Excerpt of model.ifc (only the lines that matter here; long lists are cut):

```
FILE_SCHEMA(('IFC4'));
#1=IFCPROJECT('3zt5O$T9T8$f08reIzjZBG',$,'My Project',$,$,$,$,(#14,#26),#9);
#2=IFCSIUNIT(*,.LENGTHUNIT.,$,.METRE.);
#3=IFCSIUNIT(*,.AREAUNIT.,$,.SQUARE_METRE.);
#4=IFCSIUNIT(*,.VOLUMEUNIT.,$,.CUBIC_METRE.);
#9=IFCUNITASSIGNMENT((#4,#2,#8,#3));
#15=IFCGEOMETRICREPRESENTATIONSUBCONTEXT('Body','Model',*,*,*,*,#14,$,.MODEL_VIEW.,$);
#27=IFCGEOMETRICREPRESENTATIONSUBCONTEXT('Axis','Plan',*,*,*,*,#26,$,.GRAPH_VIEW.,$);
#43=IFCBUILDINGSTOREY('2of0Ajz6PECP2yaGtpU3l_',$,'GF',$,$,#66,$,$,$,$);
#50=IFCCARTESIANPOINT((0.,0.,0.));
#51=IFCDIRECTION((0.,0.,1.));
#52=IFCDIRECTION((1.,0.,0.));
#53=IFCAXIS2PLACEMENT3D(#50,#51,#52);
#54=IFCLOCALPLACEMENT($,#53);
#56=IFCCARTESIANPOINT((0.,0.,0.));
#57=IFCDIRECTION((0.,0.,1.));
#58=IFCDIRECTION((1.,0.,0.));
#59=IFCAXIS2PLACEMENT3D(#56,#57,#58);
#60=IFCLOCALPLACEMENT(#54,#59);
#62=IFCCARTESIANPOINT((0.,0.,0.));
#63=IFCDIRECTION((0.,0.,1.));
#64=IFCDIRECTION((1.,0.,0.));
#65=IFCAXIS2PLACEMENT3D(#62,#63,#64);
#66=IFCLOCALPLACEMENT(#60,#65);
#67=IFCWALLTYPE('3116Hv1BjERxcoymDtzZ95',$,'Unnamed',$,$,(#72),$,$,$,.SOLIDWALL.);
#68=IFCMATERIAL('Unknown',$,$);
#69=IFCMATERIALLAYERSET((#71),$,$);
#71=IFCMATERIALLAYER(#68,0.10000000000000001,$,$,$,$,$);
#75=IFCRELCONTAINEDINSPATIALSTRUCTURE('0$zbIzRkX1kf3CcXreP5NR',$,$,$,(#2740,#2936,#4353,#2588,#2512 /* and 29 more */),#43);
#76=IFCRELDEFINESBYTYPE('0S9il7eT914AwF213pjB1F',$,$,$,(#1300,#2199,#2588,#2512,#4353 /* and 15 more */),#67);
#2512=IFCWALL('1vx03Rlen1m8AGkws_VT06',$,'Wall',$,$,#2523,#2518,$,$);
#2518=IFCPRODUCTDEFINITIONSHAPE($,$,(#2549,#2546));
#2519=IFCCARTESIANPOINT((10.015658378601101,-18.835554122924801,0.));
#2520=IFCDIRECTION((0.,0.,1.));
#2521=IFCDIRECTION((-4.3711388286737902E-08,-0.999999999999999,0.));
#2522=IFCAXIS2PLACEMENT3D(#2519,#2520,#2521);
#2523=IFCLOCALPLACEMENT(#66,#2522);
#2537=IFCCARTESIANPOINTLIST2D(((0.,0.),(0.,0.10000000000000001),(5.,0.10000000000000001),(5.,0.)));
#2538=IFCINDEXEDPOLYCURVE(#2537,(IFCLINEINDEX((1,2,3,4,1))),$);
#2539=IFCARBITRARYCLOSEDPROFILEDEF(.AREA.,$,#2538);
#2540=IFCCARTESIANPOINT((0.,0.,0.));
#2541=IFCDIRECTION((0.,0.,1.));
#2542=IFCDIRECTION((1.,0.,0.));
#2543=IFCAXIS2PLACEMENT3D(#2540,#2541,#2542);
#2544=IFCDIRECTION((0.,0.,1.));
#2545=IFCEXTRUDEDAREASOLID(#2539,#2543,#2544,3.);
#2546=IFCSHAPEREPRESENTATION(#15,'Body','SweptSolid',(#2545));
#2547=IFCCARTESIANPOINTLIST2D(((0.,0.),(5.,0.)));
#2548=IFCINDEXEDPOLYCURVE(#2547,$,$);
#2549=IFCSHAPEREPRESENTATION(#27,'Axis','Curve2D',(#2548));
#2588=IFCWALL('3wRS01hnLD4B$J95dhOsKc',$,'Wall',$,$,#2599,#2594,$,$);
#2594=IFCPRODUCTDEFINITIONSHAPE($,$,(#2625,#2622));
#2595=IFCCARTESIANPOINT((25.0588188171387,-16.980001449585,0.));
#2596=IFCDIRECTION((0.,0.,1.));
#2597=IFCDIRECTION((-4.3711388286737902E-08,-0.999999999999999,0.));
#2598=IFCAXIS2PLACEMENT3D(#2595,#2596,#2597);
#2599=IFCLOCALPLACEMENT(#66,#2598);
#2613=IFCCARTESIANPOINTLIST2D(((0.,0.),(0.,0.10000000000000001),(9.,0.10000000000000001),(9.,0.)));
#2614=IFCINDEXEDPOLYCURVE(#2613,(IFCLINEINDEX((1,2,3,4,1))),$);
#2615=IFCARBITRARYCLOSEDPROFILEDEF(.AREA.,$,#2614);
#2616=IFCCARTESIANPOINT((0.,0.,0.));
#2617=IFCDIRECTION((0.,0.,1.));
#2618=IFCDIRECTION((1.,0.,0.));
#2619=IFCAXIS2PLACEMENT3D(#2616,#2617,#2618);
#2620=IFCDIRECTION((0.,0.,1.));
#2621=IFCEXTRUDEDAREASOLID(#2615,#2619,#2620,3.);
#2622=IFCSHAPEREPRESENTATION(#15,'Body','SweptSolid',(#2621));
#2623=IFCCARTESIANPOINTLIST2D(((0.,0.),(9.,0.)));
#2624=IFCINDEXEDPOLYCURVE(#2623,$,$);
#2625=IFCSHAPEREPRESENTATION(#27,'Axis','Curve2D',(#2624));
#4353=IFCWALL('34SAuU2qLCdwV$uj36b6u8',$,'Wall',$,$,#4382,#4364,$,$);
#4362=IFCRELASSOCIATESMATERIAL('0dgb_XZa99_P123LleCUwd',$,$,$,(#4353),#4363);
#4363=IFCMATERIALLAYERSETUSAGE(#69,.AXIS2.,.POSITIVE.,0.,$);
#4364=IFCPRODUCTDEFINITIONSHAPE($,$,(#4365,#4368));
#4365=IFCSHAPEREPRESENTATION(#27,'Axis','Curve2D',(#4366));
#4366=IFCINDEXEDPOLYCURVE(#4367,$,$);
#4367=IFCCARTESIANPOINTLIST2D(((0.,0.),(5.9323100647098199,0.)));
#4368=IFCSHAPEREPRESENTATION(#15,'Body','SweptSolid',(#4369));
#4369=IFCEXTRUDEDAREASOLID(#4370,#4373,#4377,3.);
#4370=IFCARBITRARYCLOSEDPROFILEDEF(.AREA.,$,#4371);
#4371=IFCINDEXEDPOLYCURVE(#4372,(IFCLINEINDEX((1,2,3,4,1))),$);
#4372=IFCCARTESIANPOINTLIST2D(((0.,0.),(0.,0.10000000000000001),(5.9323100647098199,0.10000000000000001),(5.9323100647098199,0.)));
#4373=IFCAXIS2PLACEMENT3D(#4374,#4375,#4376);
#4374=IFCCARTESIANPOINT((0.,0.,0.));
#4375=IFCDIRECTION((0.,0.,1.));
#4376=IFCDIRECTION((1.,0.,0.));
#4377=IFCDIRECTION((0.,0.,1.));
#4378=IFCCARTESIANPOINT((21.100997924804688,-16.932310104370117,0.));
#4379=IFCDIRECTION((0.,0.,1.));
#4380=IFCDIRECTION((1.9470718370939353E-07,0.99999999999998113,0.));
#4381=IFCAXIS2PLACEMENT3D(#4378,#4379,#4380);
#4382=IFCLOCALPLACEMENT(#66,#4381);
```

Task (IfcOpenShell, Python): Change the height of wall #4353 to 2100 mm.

```python
import ifcopenshell
import ifcopenshell.geom
import ifcopenshell.util.representation
import ifcopenshell.util.shape
import ifcopenshell.util.unit

model = ifcopenshell.open("model.ifc")
unit_scale = ifcopenshell.util.unit.calculate_unit_scale(model)
settings = ifcopenshell.geom.settings()


def volume(element):
    """Net volume in cubic metres, openings subtracted."""
    shape = ifcopenshell.geom.create_shape(settings, element)
    return ifcopenshell.util.shape.get_volume(shape.geometry)


wall = model.by_guid("34SAuU2qLCdwV$uj36b6u8")
before = volume(wall)

body = ifcopenshell.util.representation.get_representation(wall, "Model", "Body")
solid = body.Items[0]
old_height = solid.Depth
solid.Depth = 2.1 / unit_scale
after = volume(wall)

print(f"height {old_height:g} -> {solid.Depth:g}, volume {before:.3f} -> {after:.3f} m3")

model.write("model_rev.ifc")
```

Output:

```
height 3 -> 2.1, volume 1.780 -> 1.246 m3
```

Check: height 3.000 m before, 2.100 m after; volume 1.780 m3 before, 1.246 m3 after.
